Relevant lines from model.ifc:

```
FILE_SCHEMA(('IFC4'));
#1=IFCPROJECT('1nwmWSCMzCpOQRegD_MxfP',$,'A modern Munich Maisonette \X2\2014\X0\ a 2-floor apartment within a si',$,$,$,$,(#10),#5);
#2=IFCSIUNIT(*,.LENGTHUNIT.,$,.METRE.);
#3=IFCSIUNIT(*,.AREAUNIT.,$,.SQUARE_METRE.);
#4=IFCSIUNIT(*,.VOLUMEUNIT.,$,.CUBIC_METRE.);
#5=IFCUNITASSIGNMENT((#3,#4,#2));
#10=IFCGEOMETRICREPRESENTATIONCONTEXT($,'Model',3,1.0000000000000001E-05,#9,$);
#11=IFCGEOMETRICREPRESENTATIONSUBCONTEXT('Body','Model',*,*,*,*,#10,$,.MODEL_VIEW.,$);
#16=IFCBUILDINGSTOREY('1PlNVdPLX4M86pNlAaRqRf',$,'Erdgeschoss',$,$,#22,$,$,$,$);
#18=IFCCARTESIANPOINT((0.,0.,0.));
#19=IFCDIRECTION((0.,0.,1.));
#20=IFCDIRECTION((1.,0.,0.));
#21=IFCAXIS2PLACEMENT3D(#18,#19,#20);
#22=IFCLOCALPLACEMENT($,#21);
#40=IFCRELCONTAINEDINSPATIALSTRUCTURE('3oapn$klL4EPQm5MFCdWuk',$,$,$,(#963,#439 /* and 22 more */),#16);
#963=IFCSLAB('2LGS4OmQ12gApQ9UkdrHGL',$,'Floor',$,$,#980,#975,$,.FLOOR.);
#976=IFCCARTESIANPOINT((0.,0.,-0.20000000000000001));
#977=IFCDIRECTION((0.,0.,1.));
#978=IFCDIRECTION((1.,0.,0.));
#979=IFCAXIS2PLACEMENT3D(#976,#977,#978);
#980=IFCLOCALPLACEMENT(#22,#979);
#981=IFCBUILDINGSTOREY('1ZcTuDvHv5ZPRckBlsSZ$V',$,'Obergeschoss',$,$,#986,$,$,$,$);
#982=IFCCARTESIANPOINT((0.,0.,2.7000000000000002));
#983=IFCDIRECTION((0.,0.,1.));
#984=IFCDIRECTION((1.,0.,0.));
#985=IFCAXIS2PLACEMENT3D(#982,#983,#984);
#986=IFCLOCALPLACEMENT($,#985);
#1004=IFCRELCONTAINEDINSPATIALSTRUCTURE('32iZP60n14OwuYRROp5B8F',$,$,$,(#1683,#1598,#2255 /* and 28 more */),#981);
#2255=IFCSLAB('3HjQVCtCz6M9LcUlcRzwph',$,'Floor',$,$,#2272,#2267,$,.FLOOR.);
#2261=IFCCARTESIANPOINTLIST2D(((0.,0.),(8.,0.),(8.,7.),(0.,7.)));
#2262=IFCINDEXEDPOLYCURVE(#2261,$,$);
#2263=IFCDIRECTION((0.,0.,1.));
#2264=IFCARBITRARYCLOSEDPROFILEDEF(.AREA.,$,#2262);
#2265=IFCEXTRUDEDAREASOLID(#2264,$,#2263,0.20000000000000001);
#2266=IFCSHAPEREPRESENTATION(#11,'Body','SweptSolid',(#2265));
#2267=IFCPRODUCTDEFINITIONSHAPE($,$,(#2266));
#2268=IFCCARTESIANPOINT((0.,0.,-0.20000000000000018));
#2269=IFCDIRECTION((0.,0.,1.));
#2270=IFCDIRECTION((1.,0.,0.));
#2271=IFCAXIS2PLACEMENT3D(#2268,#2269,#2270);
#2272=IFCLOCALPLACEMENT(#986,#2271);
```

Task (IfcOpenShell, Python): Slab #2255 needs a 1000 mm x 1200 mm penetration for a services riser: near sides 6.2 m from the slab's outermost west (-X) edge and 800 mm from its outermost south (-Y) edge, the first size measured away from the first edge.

```python
import numpy as np
import ifcopenshell
import ifcopenshell.api.feature
import ifcopenshell.api.geometry
import ifcopenshell.api.root
import ifcopenshell.geom
import ifcopenshell.util.placement
import ifcopenshell.util.representation
import ifcopenshell.util.shape
import ifcopenshell.util.unit

model = ifcopenshell.open("model.ifc")
unit_scale = ifcopenshell.util.unit.calculate_unit_scale(model)
settings = ifcopenshell.geom.settings()


def volume(element):
    """Net volume in cubic metres, openings subtracted."""
    shape = ifcopenshell.geom.create_shape(settings, element)
    return ifcopenshell.util.shape.get_volume(shape.geometry)


slab = model.by_id(2255)
before = volume(slab)

# Extent in the slab's own axes, in metres. The edges named are its -X and -Y sides.
slab_shape = ifcopenshell.geom.create_shape(settings, slab)
vertices = ifcopenshell.util.shape.get_vertices(slab_shape.geometry)
x_min, y_min, bottom = vertices.min(axis=0)
top = vertices[:, 2].max()

opening = ifcopenshell.api.root.create_entity(model, ifc_class="IfcOpeningElement", name="Services riser opening", predefined_type="OPENING")
context = ifcopenshell.util.representation.get_context(model, "Model", "Body", "MODEL_VIEW")
width, depth = 1, 1.2
outline = [(0.0, 0.0), (width, 0.0), (width, depth), (0.0, depth), (0.0, 0.0)]
# Overshoot both faces by 50 mm so the cut is clean.
shape = ifcopenshell.api.geometry.add_slab_representation(
    model, context=context, depth=top - bottom + 0.1, polyline=outline
)
ifcopenshell.api.geometry.assign_representation(model, product=opening, representation=shape)

matrix = ifcopenshell.util.placement.get_local_placement(slab.ObjectPlacement)
matrix[:, 3] = matrix @ np.append(np.array([x_min + 6.2, y_min + 0.8, bottom - 0.05]) / unit_scale, 1.0)
ifcopenshell.api.geometry.edit_object_placement(model, product=opening, matrix=matrix, is_si=False)
ifcopenshell.api.feature.add_feature(model, feature=opening, element=slab)

after = volume(slab)

print(f"slab volume {before:.3f} -> {after:.3f} m3")

model.write("model_updated.ifc")
```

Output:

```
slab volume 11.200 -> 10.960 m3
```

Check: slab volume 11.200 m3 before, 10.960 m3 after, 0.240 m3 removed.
